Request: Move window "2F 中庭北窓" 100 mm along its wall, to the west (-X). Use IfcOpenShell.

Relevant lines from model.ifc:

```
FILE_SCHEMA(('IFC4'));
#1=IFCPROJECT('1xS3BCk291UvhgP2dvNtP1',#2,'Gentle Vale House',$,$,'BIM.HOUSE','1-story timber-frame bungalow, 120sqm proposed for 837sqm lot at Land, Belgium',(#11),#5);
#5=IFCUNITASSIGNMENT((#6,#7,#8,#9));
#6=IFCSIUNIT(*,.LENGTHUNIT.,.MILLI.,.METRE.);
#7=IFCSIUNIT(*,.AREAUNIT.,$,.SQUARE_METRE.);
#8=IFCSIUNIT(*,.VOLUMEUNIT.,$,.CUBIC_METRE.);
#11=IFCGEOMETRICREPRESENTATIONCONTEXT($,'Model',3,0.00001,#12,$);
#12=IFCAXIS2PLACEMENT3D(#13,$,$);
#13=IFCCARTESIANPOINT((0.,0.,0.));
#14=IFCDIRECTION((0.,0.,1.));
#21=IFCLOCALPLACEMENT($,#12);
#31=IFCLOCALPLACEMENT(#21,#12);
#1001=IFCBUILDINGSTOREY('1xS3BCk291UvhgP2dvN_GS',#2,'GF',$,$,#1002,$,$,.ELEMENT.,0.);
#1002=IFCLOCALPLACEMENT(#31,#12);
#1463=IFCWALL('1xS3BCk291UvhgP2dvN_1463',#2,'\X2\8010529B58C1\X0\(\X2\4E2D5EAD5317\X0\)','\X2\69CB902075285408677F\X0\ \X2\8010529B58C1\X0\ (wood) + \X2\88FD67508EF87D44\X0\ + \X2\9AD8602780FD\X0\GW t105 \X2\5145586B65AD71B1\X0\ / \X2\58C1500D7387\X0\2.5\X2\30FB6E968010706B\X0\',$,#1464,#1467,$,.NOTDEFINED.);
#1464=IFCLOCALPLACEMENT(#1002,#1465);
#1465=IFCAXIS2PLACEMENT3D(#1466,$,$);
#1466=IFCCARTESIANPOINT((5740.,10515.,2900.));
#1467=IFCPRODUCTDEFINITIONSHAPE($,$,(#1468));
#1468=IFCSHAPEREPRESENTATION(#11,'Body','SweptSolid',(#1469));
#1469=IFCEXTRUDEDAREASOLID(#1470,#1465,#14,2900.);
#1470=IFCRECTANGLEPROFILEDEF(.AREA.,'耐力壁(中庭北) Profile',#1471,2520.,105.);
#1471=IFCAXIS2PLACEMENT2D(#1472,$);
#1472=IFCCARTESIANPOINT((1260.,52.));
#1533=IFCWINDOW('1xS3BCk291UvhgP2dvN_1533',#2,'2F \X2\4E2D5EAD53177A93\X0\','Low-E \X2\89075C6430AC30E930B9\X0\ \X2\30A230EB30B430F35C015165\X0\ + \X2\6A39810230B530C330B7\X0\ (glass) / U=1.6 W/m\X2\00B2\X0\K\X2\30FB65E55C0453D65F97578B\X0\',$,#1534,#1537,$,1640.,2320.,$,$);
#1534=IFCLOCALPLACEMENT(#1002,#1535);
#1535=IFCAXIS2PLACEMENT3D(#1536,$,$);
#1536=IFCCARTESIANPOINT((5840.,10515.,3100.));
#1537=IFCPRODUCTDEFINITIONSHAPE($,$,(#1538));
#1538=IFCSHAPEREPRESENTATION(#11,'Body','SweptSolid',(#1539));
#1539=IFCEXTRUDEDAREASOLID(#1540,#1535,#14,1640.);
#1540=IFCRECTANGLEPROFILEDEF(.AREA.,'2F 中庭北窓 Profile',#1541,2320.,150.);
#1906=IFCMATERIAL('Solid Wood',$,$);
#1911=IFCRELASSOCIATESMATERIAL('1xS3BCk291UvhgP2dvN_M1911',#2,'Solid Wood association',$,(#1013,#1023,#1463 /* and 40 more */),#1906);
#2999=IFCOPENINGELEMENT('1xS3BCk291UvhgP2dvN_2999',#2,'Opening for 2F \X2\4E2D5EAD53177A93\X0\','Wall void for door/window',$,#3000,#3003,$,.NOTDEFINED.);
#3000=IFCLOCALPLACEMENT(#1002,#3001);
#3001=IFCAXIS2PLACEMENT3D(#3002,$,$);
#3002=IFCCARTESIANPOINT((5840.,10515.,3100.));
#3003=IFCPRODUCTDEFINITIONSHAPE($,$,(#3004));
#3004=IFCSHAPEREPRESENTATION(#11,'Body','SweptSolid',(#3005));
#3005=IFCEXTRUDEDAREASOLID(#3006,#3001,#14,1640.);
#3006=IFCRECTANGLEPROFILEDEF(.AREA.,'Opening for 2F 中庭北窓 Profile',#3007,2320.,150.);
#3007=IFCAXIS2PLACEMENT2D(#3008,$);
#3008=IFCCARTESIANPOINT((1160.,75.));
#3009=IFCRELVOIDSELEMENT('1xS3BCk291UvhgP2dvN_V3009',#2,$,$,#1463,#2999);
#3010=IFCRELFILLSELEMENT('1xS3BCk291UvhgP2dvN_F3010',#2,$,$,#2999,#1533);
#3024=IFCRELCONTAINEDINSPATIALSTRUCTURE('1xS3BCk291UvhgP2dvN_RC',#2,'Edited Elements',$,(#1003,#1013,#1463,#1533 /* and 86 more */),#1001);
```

```python
import ifcopenshell
import ifcopenshell.api.geometry
import ifcopenshell.util.placement

model = ifcopenshell.open("model.ifc")

window = model.by_guid("1xS3BCk291UvhgP2dvN_1533")
opening = window.FillsVoids[0].RelatingOpeningElement
wall = opening.VoidsElements[0].RelatingBuildingElement

wall_matrix = ifcopenshell.util.placement.get_local_placement(wall.ObjectPlacement)
shift = wall_matrix[:3, 0] * -100.0
before = ifcopenshell.util.placement.get_local_placement(window.ObjectPlacement)[:3, 3].copy()

# The window is not placed relative to its opening, so move both.
for product in (opening, window):
    matrix = ifcopenshell.util.placement.get_local_placement(product.ObjectPlacement)
    matrix[:3, 3] += shift
    ifcopenshell.api.geometry.edit_object_placement(model, product=product, matrix=matrix, is_si=False)

after = ifcopenshell.util.placement.get_local_placement(window.ObjectPlacement)[:3, 3]
print("window moved by", (after - before).round(3) + 0.0)

model.write("model_rev.ifc")
```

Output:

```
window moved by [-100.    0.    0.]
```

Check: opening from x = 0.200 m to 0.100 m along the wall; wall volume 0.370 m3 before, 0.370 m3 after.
